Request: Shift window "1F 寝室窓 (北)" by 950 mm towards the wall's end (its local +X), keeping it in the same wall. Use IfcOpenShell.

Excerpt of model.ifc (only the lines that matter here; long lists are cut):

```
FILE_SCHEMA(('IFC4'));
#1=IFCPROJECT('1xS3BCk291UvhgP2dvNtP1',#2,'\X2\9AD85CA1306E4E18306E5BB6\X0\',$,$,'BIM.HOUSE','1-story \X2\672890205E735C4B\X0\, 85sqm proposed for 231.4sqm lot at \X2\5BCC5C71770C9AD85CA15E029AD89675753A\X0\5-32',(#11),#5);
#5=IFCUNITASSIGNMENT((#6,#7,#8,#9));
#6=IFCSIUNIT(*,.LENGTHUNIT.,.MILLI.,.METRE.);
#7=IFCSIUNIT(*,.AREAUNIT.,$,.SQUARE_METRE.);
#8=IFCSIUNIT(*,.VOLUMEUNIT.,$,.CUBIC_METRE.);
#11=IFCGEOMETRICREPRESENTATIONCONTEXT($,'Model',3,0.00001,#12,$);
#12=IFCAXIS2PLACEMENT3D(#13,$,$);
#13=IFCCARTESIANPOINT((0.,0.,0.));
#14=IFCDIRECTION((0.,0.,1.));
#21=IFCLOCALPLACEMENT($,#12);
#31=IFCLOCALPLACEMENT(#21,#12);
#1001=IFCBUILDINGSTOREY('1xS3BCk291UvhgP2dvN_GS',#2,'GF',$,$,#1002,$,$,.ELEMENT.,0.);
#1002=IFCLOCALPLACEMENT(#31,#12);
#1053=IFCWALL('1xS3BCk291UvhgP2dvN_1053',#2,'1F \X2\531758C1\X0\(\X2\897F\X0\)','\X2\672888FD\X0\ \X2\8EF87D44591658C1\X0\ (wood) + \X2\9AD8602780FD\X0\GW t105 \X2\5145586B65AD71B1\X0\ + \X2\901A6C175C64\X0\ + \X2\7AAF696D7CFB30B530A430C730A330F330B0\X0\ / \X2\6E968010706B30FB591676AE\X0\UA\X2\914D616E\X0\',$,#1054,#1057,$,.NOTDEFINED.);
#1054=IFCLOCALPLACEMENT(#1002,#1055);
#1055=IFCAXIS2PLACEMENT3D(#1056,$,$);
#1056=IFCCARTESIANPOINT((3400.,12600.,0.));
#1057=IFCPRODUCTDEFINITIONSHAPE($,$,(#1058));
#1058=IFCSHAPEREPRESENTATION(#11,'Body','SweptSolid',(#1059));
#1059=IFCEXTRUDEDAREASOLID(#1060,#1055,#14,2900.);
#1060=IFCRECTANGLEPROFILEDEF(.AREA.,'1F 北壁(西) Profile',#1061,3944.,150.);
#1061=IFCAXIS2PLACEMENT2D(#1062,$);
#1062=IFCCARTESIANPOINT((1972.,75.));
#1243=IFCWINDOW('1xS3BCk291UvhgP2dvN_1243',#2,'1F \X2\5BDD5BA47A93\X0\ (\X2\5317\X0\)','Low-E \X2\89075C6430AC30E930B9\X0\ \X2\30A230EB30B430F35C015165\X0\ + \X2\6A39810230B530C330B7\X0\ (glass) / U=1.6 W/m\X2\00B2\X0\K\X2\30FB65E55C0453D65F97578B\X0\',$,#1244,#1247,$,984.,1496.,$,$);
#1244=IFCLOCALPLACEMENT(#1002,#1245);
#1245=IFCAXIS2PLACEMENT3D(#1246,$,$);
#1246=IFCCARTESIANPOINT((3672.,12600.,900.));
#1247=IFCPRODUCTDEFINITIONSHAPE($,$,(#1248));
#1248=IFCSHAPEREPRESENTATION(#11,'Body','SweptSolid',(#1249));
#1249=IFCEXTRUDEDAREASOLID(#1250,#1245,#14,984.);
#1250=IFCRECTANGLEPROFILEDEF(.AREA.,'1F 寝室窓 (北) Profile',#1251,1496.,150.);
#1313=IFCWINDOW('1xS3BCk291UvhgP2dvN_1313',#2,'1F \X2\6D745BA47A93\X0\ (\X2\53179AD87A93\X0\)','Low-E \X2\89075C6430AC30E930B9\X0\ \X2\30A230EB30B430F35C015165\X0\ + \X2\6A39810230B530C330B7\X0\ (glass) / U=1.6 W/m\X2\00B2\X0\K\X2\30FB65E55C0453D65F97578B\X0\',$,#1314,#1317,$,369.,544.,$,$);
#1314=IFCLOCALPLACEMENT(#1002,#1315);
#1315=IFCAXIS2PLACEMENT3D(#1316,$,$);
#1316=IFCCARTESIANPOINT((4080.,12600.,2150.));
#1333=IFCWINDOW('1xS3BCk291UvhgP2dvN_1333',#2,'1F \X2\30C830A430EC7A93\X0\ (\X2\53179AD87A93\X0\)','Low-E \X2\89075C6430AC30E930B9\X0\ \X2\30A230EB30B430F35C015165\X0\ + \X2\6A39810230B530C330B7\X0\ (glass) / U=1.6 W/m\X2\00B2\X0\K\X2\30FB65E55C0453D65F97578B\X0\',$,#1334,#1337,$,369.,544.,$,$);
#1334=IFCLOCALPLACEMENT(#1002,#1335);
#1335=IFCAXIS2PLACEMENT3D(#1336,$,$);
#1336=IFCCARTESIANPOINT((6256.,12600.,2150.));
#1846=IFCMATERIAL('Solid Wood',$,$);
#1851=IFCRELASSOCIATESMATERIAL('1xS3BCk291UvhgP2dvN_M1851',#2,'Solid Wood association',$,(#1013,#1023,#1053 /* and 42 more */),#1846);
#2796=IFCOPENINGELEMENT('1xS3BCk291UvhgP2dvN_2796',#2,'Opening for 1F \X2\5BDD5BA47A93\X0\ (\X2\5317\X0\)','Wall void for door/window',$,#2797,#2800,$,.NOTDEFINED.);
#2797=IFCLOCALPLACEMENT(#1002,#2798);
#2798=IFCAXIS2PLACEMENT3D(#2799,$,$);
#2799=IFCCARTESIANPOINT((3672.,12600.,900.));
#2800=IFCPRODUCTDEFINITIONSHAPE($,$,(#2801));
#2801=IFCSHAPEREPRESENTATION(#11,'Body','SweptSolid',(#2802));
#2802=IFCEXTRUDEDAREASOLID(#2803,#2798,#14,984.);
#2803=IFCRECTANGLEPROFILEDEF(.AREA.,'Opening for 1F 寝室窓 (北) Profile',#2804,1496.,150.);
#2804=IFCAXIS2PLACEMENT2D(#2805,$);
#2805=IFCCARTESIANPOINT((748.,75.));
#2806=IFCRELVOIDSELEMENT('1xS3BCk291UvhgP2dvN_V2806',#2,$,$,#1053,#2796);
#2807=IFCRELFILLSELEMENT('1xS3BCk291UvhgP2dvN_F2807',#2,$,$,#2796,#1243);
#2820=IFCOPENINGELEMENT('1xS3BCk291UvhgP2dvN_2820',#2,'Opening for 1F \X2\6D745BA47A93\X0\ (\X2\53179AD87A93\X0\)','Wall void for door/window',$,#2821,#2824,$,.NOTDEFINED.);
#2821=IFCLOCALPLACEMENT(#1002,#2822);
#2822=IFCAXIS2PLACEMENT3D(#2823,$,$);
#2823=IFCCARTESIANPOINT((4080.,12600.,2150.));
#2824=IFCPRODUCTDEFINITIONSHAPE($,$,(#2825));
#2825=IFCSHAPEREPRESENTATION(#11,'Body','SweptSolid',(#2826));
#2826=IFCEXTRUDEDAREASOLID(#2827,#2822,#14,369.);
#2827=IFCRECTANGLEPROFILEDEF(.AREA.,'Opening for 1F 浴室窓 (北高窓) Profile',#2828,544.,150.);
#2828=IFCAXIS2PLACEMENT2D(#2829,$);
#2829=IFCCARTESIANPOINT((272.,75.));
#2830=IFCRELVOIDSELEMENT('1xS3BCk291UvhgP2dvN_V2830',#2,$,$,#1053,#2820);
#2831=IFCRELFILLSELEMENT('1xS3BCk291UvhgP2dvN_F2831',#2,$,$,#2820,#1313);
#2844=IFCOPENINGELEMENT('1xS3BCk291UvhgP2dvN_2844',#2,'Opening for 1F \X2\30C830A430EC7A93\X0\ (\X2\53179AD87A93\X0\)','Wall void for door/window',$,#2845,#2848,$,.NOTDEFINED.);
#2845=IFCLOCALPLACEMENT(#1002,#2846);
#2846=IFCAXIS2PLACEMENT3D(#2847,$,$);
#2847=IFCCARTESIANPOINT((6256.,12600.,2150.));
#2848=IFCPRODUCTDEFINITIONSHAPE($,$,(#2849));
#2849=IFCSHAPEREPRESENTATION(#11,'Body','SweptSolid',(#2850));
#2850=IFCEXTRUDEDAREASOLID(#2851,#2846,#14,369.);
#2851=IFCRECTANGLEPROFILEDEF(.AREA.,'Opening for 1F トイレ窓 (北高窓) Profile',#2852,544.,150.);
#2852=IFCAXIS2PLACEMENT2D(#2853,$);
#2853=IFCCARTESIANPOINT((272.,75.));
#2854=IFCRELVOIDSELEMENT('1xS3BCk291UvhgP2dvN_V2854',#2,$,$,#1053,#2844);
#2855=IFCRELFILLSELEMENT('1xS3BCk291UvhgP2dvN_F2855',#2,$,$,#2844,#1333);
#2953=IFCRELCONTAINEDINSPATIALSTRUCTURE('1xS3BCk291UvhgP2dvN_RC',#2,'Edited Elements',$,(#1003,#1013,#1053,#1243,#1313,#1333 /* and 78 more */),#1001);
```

```python
import ifcopenshell
import ifcopenshell.api.geometry
import ifcopenshell.util.placement

model = ifcopenshell.open("model.ifc")

window = model.by_guid("1xS3BCk291UvhgP2dvN_1243")
opening = window.FillsVoids[0].RelatingOpeningElement
wall = opening.VoidsElements[0].RelatingBuildingElement

wall_matrix = ifcopenshell.util.placement.get_local_placement(wall.ObjectPlacement)
shift = wall_matrix[:3, 0] * 950.0
before = ifcopenshell.util.placement.get_local_placement(window.ObjectPlacement)[:3, 3].copy()

# The window is not placed relative to its opening, so move both.
for product in (opening, window):
    matrix = ifcopenshell.util.placement.get_local_placement(product.ObjectPlacement)
    matrix[:3, 3] += shift
    ifcopenshell.api.geometry.edit_object_placement(model, product=product, matrix=matrix, is_si=False)

after = ifcopenshell.util.placement.get_local_placement(window.ObjectPlacement)[:3, 3]
print("window moved by", (after - before).round(3) + 0.0)

model.write("model_edited.ifc")
```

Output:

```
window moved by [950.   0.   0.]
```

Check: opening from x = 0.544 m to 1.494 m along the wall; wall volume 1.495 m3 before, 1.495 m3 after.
